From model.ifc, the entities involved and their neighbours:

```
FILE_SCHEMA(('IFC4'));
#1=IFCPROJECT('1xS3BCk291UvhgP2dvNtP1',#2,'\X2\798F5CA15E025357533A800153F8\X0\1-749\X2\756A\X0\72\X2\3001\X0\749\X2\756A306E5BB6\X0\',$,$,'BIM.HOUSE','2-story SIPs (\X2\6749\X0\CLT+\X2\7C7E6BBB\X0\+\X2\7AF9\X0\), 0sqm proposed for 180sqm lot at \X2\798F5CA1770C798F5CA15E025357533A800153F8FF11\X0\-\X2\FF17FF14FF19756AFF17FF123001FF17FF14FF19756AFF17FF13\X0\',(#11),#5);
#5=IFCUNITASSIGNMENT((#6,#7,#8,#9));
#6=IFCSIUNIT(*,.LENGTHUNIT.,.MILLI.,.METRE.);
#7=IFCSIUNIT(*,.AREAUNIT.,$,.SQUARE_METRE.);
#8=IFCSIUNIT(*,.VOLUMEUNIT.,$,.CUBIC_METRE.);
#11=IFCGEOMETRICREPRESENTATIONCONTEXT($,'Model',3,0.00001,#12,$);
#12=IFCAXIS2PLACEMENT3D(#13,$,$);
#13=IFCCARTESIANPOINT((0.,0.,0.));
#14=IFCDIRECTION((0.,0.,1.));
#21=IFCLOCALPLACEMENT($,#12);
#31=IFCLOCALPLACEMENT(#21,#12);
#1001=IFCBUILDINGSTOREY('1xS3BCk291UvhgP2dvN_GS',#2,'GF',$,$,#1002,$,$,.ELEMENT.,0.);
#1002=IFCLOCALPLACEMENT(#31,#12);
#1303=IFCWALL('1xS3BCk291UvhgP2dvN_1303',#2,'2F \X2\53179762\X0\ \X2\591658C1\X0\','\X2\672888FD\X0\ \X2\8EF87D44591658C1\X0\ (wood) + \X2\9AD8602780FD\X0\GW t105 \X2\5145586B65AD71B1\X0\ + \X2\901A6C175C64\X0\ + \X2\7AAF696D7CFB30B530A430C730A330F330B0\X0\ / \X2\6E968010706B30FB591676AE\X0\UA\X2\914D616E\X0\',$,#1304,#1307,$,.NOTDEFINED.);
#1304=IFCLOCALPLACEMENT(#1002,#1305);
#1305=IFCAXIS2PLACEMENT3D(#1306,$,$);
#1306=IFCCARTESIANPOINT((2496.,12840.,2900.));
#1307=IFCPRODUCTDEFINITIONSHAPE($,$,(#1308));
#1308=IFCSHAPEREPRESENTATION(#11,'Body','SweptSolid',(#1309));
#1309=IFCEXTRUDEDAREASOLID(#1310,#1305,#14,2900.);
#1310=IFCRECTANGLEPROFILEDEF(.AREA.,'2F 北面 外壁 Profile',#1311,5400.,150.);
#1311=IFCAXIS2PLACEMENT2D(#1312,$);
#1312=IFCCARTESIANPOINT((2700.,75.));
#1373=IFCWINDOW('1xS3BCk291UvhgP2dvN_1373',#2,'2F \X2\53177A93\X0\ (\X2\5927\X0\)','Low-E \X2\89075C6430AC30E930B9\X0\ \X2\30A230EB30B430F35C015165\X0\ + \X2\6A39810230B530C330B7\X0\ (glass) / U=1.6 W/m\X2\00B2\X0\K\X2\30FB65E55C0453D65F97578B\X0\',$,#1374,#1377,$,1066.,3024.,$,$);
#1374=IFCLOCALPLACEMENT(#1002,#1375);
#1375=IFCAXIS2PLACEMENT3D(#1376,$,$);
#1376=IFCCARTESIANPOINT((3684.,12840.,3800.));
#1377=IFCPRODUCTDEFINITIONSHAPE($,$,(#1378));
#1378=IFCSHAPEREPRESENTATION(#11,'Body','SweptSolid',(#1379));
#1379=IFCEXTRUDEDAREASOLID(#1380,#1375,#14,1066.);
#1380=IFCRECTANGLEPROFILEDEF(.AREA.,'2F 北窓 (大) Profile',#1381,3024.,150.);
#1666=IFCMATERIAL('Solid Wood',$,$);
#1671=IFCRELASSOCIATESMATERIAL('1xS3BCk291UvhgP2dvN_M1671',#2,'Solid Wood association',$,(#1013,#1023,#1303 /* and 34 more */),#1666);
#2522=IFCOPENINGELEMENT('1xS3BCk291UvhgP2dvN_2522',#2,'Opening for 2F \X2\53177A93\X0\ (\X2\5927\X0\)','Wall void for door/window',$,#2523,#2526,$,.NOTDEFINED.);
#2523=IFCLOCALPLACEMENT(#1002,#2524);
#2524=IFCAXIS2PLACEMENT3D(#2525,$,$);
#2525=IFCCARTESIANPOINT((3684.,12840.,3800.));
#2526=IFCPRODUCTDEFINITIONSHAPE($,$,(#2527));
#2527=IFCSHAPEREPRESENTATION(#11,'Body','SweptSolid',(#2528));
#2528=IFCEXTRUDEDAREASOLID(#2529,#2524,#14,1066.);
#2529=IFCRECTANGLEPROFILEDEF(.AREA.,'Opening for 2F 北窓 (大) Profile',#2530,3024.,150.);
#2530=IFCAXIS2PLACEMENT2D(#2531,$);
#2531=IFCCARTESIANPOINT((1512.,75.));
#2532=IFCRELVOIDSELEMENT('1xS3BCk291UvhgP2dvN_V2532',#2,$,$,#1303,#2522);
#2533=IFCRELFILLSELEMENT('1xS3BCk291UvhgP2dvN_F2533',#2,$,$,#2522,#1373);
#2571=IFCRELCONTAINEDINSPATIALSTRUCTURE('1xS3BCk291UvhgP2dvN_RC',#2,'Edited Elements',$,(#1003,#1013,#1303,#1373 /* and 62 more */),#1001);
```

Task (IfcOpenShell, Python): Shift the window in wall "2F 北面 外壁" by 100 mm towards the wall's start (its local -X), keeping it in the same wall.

```python
import ifcopenshell
import ifcopenshell.api.geometry
import ifcopenshell.util.placement

model = ifcopenshell.open("model.ifc")

window = model.by_guid("1xS3BCk291UvhgP2dvN_1373")
opening = window.FillsVoids[0].RelatingOpeningElement
wall = opening.VoidsElements[0].RelatingBuildingElement

wall_matrix = ifcopenshell.util.placement.get_local_placement(wall.ObjectPlacement)
shift = wall_matrix[:3, 0] * -100.0
before = ifcopenshell.util.placement.get_local_placement(window.ObjectPlacement)[:3, 3].copy()

# The window is not placed relative to its opening, so move both.
for product in (opening, window):
    matrix = ifcopenshell.util.placement.get_local_placement(product.ObjectPlacement)
    matrix[:3, 3] += shift
    ifcopenshell.api.geometry.edit_object_placement(model, product=product, matrix=matrix, is_si=False)

after = ifcopenshell.util.placement.get_local_placement(window.ObjectPlacement)[:3, 3]
print("window moved by", (after - before).round(3) + 0.0)

model.write("model-out.ifc")
```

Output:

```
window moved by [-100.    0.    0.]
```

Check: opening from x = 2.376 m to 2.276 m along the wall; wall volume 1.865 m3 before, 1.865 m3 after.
